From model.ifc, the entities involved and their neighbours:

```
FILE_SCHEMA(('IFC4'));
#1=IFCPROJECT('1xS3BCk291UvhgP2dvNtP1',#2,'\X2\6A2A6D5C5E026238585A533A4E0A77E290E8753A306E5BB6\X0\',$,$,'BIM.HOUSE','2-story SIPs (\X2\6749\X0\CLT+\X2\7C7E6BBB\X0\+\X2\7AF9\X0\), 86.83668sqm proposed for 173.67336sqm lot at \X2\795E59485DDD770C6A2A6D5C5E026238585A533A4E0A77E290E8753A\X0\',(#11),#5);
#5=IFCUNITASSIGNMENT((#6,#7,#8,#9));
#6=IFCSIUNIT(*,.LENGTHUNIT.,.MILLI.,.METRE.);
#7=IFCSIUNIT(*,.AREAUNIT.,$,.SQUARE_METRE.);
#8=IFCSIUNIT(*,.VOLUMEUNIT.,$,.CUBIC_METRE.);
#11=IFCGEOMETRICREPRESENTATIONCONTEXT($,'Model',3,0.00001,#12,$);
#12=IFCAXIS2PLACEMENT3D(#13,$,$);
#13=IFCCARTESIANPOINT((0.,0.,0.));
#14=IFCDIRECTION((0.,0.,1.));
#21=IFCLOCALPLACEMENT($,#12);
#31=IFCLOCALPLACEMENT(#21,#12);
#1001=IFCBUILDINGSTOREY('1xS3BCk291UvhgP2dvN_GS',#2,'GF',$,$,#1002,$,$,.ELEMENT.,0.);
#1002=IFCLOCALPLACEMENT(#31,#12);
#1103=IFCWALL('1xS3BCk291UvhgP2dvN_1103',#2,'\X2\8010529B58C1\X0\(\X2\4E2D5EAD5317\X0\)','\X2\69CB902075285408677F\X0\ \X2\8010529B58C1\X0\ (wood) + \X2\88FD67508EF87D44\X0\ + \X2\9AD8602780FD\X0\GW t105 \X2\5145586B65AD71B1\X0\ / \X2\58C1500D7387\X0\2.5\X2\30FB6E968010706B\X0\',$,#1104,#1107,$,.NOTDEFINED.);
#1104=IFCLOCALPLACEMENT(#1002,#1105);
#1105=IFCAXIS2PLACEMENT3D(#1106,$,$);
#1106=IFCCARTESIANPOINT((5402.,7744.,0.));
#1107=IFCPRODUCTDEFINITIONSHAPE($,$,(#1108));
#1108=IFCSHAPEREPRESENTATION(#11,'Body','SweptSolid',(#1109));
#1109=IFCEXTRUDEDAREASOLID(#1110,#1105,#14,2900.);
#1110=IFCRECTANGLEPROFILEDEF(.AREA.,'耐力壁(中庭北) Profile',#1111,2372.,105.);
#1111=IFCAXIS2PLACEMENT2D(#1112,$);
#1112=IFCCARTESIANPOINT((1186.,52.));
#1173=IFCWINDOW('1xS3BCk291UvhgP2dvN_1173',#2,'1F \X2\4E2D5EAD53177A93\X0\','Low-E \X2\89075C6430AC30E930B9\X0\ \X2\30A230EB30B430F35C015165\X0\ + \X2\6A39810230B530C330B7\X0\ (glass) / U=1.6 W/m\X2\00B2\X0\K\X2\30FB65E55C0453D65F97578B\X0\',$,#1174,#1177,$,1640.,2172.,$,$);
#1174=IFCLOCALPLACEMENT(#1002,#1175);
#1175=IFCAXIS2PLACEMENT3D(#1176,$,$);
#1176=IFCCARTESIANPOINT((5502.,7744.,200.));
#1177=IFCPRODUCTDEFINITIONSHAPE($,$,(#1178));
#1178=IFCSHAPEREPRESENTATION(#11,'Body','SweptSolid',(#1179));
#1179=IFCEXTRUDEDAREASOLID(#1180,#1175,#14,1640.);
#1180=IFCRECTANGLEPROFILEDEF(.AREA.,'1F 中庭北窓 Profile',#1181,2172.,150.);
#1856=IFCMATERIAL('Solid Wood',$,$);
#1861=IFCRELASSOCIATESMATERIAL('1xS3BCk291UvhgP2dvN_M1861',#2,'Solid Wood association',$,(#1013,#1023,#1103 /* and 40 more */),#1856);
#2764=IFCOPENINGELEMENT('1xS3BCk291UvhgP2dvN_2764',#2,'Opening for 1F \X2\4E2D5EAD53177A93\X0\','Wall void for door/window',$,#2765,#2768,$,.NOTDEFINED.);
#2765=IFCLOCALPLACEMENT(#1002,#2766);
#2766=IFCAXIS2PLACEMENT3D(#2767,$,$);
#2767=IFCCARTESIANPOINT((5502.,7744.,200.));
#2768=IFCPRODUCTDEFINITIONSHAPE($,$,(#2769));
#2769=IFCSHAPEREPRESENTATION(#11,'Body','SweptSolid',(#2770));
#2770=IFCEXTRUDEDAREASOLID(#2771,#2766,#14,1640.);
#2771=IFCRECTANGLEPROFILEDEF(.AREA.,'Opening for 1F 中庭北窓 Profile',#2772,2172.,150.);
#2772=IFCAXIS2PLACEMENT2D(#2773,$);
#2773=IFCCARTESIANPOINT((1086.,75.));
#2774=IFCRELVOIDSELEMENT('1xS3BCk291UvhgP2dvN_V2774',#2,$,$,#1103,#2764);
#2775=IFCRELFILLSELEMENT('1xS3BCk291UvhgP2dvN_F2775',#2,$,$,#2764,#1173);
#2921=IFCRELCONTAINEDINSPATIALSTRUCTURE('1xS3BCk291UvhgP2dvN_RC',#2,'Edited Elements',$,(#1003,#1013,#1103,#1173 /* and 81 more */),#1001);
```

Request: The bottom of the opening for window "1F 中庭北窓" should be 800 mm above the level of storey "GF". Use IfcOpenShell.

```python
import numpy as np
import ifcopenshell
import ifcopenshell.api.geometry
import ifcopenshell.geom
import ifcopenshell.util.element
import ifcopenshell.util.placement
import ifcopenshell.util.shape
import ifcopenshell.util.unit

model = ifcopenshell.open("model.ifc")
unit_scale = ifcopenshell.util.unit.calculate_unit_scale(model)

window = model.by_guid("1xS3BCk291UvhgP2dvN_1173")
opening = window.FillsVoids[0].RelatingOpeningElement
storey = ifcopenshell.util.element.get_container(window, ifc_class="IfcBuildingStorey")
level = ifcopenshell.util.placement.get_local_placement(storey.ObjectPlacement)[2, 3]

# The opening's origin need not be at the sill, so measure its lowest point.
shape = ifcopenshell.geom.create_shape(ifcopenshell.geom.settings(), opening)
bottom = ifcopenshell.util.shape.get_shape_bottom_elevation(shape, shape.geometry) / unit_scale
dz = level + 0.8 / unit_scale - bottom

shift = np.array([0.0, 0.0, dz])
# The window is not placed relative to its opening, so move both.
for product in (opening, window):
    matrix = ifcopenshell.util.placement.get_local_placement(product.ObjectPlacement)
    matrix[:3, 3] += shift
    ifcopenshell.api.geometry.edit_object_placement(model, product=product, matrix=matrix, is_si=False)

print(f"moved by {dz * unit_scale:+.3f} m")

model.write("model_updated.ifc")
```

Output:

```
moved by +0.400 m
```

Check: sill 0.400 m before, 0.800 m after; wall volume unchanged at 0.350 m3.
